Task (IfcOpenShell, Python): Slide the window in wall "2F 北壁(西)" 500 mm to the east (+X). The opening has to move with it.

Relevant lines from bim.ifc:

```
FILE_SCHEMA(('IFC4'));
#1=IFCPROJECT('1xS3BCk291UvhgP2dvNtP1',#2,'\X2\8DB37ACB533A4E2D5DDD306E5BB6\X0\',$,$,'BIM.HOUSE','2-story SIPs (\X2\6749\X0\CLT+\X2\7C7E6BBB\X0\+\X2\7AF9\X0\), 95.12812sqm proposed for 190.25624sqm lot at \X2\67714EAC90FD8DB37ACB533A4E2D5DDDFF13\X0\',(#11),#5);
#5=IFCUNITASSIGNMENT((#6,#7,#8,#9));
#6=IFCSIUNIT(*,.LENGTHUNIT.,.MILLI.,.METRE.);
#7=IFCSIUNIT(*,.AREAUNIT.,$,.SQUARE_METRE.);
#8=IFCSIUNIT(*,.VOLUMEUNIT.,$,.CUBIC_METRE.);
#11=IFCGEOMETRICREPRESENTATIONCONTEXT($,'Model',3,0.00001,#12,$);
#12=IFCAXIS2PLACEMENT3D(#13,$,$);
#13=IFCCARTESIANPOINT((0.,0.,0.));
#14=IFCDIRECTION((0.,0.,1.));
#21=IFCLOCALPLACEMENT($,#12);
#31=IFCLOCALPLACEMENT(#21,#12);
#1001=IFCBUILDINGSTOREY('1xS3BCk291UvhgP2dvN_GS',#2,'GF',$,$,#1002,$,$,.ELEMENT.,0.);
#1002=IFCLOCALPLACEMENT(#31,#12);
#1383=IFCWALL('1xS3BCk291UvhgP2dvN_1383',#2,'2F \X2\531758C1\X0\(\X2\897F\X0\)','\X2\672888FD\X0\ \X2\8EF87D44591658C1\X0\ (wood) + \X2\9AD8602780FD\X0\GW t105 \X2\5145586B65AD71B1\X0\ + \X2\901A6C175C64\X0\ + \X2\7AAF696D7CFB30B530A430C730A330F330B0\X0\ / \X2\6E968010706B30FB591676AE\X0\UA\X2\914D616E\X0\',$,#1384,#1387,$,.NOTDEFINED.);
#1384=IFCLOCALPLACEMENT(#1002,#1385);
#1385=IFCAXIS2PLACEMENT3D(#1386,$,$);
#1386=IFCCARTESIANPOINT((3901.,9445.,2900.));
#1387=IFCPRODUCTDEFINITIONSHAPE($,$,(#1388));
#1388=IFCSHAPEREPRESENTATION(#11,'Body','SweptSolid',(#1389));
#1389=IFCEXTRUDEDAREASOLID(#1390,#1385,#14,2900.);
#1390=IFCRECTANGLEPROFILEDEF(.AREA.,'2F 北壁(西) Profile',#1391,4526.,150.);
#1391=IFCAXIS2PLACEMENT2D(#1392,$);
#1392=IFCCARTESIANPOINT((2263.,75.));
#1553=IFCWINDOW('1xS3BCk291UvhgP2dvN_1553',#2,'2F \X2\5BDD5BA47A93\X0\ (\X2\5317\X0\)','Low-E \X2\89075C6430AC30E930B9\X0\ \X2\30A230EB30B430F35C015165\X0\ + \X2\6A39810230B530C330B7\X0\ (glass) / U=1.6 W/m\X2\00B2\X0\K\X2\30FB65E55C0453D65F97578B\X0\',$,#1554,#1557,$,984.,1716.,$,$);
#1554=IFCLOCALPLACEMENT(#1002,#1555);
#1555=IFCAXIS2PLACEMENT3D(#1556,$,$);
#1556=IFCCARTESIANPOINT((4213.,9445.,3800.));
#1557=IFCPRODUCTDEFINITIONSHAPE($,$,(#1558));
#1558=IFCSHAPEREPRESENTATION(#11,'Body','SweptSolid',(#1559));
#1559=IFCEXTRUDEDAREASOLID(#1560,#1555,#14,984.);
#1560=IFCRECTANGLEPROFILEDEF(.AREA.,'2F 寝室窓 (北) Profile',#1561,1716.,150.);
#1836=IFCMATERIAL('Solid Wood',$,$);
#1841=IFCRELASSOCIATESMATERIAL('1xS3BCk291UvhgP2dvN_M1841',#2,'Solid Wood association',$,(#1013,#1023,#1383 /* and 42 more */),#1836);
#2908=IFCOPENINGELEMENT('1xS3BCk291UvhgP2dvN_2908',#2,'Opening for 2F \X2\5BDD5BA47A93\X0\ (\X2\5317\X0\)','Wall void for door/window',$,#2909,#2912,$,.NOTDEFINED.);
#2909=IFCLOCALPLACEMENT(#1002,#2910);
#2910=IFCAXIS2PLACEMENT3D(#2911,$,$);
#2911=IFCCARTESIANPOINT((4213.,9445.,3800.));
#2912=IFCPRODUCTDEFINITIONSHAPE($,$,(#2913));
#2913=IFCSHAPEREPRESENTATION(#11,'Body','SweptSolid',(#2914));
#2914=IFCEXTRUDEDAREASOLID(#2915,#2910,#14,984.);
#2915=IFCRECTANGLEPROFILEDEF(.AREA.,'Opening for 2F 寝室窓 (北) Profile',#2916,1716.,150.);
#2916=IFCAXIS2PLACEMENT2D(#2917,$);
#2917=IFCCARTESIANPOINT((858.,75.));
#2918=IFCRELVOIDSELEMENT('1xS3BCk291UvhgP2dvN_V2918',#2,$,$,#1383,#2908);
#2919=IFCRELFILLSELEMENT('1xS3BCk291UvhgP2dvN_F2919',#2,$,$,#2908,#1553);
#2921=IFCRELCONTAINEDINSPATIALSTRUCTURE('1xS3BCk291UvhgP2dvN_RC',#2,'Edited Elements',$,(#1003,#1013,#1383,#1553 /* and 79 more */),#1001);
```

```python
import ifcopenshell
import ifcopenshell.api.geometry
import ifcopenshell.util.placement

model = ifcopenshell.open("bim.ifc")

window = model.by_guid("1xS3BCk291UvhgP2dvN_1553")
opening = window.FillsVoids[0].RelatingOpeningElement
wall = opening.VoidsElements[0].RelatingBuildingElement

wall_matrix = ifcopenshell.util.placement.get_local_placement(wall.ObjectPlacement)
shift = wall_matrix[:3, 0] * 500.0
before = ifcopenshell.util.placement.get_local_placement(window.ObjectPlacement)[:3, 3].copy()

# The window is not placed relative to its opening, so move both.
for product in (opening, window):
    matrix = ifcopenshell.util.placement.get_local_placement(product.ObjectPlacement)
    matrix[:3, 3] += shift
    ifcopenshell.api.geometry.edit_object_placement(model, product=product, matrix=matrix, is_si=False)

after = ifcopenshell.util.placement.get_local_placement(window.ObjectPlacement)[:3, 3]
print("window moved by", (after - before).round(3) + 0.0)

model.write("bim_updated.ifc")
```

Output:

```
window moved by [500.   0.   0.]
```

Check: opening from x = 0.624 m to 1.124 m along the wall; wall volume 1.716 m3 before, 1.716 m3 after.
